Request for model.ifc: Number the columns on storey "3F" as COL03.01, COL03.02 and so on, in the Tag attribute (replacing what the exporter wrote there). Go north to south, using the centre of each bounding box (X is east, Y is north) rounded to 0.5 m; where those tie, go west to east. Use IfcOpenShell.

First a look at what the model holds.

```python
import ifcopenshell
import ifcopenshell.util.element
import ifcopenshell.util.placement

model = ifcopenshell.open("model.ifc")
print(model.schema)
storey = next(s for s in model.by_type("IfcBuildingStorey") if s.Name == "3F")
columns = [e for e in ifcopenshell.util.element.get_decomposition(storey) if e.is_a("IfcColumn")]
for e in sorted(columns, key=lambda e: e.id()):
    origin = ifcopenshell.util.placement.get_local_placement(e.ObjectPlacement)[:3, 3]
    print(e.id(), e.Tag, e.Name, origin.round(2) + 0.0, sep=" | ")
```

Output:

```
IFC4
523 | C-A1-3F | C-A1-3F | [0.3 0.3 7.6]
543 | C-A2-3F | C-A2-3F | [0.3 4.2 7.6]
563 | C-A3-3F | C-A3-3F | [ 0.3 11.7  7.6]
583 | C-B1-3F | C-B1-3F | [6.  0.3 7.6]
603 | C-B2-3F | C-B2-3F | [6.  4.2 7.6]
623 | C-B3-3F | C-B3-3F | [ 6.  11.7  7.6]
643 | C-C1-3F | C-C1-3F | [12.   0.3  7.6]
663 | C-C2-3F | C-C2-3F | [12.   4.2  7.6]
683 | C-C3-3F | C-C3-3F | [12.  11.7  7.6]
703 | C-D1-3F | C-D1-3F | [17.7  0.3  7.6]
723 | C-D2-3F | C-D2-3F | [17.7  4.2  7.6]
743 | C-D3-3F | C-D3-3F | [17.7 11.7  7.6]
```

```python
import ifcopenshell
import ifcopenshell.geom
import ifcopenshell.util.element
import ifcopenshell.util.shape

model = ifcopenshell.open("model.ifc")
settings = ifcopenshell.geom.settings()
settings.set("use-world-coords", True)


def centre(element):
    shape = ifcopenshell.geom.create_shape(settings, element)
    return ifcopenshell.util.shape.get_bbox_centroid(shape.geometry)


storey = next(s for s in model.by_type("IfcBuildingStorey") if s.Name == "3F")
columns = [e for e in ifcopenshell.util.element.get_decomposition(storey) if e.is_a("IfcColumn")]

# Insertion points can sit at a corner or the storey origin, so sort by the geometry (in metres).
centres = {e: centre(e) for e in columns}
columns.sort(key=lambda e: (-round(centres[e][1] / 0.5), centres[e][0]))

for i, e in enumerate(columns, start=1):
    number = f"COL03.{i:02d}"
    e.Tag = number
    print(e.id(), number)

model.write("model_rev.ifc")
```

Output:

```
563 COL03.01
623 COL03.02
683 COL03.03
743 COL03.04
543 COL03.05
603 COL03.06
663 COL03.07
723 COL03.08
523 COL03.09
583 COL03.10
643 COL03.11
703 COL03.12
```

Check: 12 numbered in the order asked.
